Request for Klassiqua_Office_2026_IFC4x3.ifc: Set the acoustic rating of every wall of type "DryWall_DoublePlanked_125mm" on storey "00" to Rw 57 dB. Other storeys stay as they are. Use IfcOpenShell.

First a look at what the model holds.

```python
import ifcopenshell
import ifcopenshell.util.element

model = ifcopenshell.open("Klassiqua_Office_2026_IFC4x3.ifc")
print(model.schema)
storey = next(s for s in model.by_type("IfcBuildingStorey") if s.Name == "00")
walls = [e for e in ifcopenshell.util.element.get_decomposition(storey) if e.is_a("IfcWall")]
seen = {}
for e in walls:
    element_type = ifcopenshell.util.element.get_type(e)
    key = (element_type.Name if element_type != e and element_type else None, ifcopenshell.util.element.get_pset(e, "Pset_WallCommon", "AcousticRating"))
    seen[key] = seen.get(key, 0) + 1
for (name, value), count in sorted(seen.items(), key=str):
    print(count, "x", name, "|", value)
```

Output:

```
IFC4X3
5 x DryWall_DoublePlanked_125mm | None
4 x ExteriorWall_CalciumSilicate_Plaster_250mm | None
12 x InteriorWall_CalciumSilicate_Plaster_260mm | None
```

```python
import ifcopenshell
import ifcopenshell.api.pset
import ifcopenshell.util.element

model = ifcopenshell.open("Klassiqua_Office_2026_IFC4x3.ifc")

storey = next(s for s in model.by_type("IfcBuildingStorey") if s.Name == "00")
walls = [e for e in ifcopenshell.util.element.get_decomposition(storey) if e.is_a("IfcWall")]

count = 0
for e in walls:
    element_type = ifcopenshell.util.element.get_type(e)
    if element_type in (None, e) or element_type.Name != "DryWall_DoublePlanked_125mm":
        continue
    # add_pset returns the element's existing set when there is one.
    pset = ifcopenshell.api.pset.add_pset(model, product=e, name="Pset_WallCommon")
    ifcopenshell.api.pset.edit_pset(model, pset=pset, properties={"AcousticRating": "Rw 57 dB"})
    count += 1

print(count, "walls updated")

model.write("Klassiqua_Office_2026_IFC4x3_updated.ifc")
```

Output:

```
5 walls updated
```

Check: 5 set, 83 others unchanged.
